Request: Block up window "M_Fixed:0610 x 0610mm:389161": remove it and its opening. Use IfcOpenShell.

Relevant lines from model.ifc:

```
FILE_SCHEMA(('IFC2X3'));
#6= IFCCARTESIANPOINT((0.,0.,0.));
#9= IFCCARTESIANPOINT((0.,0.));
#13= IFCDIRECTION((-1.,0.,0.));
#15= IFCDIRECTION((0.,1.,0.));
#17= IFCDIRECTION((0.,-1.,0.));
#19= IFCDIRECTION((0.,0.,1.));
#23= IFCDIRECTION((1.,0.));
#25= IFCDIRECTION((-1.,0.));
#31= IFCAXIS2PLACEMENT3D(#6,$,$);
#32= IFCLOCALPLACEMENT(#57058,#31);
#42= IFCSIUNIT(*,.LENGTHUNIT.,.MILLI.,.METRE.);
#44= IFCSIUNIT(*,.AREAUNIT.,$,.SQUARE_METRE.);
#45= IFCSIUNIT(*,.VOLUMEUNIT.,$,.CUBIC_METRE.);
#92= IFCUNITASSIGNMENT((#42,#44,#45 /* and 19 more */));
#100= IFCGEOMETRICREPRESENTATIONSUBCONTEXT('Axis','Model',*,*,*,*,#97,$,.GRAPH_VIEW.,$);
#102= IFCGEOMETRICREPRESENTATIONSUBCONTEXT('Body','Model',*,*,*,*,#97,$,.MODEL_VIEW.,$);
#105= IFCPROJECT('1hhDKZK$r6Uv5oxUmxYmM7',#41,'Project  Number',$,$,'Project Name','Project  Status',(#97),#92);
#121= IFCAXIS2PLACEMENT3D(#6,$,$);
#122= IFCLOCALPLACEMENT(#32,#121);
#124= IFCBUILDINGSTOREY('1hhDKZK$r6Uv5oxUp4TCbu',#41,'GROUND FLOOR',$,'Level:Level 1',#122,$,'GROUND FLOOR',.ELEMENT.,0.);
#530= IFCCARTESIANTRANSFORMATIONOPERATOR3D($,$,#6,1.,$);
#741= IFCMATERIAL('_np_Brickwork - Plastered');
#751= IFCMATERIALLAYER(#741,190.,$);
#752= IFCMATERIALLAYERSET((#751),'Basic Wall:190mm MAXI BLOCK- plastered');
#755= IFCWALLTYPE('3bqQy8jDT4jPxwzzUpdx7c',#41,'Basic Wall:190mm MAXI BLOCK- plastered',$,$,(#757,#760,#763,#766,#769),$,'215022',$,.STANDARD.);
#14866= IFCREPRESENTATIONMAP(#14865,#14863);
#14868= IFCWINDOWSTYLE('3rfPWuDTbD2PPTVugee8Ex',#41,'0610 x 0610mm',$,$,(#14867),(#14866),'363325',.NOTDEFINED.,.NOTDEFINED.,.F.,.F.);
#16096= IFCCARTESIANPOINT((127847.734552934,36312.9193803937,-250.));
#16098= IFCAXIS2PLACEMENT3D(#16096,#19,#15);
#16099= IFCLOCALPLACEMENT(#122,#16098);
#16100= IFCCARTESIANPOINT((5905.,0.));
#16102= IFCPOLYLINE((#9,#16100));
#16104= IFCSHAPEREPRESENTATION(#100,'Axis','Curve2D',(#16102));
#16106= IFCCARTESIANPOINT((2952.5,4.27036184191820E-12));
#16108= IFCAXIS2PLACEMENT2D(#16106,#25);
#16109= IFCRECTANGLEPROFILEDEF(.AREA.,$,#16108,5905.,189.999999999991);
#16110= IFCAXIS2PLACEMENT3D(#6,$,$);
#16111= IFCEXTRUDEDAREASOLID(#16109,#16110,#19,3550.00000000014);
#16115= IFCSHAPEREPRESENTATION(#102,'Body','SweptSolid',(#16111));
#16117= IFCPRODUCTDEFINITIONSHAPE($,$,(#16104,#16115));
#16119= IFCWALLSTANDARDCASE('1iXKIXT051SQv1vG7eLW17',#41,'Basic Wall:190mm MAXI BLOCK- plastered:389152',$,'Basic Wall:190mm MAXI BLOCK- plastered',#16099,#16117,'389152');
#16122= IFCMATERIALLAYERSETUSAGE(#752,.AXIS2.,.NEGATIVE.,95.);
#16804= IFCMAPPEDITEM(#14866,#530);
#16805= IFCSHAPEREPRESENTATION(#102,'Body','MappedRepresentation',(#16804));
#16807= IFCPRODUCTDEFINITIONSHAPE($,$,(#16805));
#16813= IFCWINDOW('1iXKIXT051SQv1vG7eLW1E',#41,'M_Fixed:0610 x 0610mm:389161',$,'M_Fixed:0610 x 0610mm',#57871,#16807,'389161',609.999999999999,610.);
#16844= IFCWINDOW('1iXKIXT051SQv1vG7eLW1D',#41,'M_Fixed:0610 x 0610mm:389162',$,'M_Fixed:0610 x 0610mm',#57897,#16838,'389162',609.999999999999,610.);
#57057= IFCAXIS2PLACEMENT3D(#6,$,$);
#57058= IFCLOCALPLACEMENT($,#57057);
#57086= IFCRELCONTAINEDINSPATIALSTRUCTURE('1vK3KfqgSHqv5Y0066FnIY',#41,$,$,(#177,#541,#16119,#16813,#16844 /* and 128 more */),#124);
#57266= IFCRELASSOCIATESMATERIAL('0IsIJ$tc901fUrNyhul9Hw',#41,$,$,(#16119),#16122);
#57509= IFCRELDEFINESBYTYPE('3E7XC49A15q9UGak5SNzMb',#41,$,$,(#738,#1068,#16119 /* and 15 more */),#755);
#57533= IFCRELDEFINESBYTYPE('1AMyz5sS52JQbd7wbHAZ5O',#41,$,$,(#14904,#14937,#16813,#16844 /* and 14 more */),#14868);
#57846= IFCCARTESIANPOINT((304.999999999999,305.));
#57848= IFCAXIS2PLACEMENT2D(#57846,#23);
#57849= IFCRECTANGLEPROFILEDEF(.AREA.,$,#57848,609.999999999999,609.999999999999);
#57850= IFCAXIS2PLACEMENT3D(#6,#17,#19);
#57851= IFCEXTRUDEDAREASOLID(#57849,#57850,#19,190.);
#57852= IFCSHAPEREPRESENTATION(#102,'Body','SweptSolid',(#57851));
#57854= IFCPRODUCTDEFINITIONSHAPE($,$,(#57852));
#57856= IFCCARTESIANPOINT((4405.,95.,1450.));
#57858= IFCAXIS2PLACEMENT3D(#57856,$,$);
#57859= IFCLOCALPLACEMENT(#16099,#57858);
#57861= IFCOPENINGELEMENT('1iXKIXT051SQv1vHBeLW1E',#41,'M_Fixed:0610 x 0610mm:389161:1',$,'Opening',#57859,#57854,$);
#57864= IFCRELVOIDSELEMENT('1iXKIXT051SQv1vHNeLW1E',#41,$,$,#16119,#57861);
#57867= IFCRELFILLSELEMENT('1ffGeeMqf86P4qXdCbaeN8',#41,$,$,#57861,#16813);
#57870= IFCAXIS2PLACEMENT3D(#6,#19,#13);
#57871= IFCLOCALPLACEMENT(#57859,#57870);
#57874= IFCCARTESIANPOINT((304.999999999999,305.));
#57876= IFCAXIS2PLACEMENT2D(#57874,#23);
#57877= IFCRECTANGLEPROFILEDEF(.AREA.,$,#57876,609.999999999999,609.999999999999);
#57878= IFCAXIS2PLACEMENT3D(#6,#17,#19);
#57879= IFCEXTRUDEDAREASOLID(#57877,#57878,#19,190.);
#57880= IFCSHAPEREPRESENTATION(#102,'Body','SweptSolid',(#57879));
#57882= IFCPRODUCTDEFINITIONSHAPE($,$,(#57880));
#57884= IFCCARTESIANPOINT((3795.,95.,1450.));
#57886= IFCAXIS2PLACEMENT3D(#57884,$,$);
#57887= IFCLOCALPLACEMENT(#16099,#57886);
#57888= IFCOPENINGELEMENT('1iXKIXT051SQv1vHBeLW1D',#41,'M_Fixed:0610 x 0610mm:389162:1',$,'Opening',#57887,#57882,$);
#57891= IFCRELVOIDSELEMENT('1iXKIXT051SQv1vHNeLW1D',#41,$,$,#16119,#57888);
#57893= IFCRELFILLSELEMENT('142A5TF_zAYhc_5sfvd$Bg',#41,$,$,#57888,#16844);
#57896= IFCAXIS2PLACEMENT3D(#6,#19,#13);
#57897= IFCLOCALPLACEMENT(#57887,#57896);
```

```python
import ifcopenshell
import ifcopenshell.api.feature
import ifcopenshell.api.root
import ifcopenshell.geom
import ifcopenshell.util.shape

model = ifcopenshell.open("model.ifc")
settings = ifcopenshell.geom.settings()


def volume(element):
    """Net volume in cubic metres, openings subtracted."""
    shape = ifcopenshell.geom.create_shape(settings, element)
    return ifcopenshell.util.shape.get_volume(shape.geometry)


window = model.by_id(16813)
opening = window.FillsVoids[0].RelatingOpeningElement
wall = opening.VoidsElements[0].RelatingBuildingElement
before = volume(wall)

ifcopenshell.api.root.remove_product(model, product=window)
ifcopenshell.api.feature.remove_feature(model, feature=opening)

after = volume(wall)

print(f"wall volume {before:.3f} -> {after:.3f} m3")

model.write("model-out.ifc")
```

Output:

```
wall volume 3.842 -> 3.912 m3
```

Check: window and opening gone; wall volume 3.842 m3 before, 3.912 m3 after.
